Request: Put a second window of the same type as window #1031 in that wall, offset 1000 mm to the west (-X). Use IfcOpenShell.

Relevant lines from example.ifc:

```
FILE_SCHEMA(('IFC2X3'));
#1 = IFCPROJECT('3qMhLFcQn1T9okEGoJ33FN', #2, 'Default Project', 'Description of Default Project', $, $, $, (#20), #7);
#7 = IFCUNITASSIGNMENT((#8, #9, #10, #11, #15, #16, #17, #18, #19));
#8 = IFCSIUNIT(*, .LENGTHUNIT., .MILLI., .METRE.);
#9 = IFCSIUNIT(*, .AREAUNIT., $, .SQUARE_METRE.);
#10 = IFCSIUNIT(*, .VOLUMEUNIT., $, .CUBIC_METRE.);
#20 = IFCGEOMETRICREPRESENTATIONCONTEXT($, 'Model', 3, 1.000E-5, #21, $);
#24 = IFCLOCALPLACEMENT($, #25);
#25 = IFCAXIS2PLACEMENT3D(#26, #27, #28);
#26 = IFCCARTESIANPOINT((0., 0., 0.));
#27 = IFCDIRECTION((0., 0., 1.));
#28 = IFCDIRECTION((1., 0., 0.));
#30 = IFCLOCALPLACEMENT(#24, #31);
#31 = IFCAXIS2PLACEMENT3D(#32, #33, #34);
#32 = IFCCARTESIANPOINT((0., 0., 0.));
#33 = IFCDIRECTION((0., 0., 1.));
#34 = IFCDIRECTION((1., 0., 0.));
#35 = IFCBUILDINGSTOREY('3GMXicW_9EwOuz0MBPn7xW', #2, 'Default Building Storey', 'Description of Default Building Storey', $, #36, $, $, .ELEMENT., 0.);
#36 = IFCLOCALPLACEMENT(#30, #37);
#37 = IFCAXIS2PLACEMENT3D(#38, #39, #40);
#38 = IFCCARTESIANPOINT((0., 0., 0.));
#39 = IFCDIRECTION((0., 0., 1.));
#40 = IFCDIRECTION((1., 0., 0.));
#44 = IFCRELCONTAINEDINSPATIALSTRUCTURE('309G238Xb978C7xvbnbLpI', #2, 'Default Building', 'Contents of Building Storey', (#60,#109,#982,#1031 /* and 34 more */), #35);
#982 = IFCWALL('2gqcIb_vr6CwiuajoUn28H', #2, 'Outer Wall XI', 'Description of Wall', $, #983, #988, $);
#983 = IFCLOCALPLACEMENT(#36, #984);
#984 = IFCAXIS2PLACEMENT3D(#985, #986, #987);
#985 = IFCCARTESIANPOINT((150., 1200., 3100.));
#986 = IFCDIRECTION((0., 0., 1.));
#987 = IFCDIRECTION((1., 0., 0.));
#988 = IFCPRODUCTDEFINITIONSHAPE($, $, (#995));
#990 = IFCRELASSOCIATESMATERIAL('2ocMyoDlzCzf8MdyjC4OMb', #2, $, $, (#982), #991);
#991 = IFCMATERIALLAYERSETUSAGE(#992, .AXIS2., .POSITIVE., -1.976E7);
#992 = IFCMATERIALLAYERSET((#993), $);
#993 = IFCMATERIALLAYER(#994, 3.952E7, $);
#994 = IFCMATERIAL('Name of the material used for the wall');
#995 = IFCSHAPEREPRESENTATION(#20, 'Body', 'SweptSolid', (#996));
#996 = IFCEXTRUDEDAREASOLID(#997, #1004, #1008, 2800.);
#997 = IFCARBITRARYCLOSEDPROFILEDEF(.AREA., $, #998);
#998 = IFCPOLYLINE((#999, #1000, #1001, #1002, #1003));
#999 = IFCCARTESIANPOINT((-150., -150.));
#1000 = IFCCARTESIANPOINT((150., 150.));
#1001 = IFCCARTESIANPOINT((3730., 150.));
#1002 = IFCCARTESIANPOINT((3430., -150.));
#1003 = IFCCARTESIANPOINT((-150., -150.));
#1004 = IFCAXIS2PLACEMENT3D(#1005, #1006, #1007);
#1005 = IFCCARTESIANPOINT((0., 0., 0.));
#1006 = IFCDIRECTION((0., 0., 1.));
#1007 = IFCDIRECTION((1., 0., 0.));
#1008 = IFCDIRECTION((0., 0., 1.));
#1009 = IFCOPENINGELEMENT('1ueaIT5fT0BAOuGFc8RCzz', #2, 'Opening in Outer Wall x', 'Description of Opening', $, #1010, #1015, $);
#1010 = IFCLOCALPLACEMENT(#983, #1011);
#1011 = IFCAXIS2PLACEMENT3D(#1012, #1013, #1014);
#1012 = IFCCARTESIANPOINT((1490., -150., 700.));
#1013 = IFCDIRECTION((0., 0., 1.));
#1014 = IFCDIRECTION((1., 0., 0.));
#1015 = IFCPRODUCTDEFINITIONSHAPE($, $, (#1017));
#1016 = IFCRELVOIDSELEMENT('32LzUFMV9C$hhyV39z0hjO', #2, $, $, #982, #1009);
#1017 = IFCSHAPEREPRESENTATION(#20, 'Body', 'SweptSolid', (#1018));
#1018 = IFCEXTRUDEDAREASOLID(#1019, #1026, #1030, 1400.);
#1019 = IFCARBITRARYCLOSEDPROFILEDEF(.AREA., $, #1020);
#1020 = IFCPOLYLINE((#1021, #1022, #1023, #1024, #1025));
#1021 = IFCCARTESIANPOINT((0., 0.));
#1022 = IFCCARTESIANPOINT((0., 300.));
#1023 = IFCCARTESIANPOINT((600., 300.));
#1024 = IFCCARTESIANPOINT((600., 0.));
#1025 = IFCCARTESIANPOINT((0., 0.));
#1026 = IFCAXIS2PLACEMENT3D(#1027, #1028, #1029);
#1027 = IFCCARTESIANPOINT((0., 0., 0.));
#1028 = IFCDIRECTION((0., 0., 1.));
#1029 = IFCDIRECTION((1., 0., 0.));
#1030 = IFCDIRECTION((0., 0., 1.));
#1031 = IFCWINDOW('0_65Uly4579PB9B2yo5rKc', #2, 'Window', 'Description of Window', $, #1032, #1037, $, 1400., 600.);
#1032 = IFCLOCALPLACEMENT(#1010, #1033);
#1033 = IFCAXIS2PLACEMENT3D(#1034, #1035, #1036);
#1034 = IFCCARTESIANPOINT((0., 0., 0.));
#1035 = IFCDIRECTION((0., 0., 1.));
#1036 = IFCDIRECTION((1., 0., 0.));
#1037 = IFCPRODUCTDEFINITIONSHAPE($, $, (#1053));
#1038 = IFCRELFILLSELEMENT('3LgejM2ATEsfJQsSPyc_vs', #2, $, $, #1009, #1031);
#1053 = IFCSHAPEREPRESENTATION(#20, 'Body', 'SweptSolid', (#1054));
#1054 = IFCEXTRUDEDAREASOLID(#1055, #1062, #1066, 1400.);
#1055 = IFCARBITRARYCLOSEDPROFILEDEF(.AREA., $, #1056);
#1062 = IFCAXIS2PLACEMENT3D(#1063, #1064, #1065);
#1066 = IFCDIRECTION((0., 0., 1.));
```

```python
import ifcopenshell
import ifcopenshell.api.feature
import ifcopenshell.api.geometry
import ifcopenshell.api.root
import ifcopenshell.geom
import ifcopenshell.util.element
import ifcopenshell.util.placement
import ifcopenshell.util.shape
import ifcopenshell.util.unit

model = ifcopenshell.open("example.ifc")
unit_scale = ifcopenshell.util.unit.calculate_unit_scale(model)
settings = ifcopenshell.geom.settings()


def volume(element):
    """Net volume in cubic metres, openings subtracted."""
    shape = ifcopenshell.geom.create_shape(settings, element)
    return ifcopenshell.util.shape.get_volume(shape.geometry)


def reuse_history(source, copy):
    """copy_class also copies each property set's owner history, people and application; keep the originals."""
    for rel in copy.IsDefinedBy:
        if rel.is_a("IfcRelDefinesByProperties") and (history := rel.RelatingPropertyDefinition.OwnerHistory):
            rel.RelatingPropertyDefinition.OwnerHistory = source.OwnerHistory
            ifcopenshell.util.element.remove_deep2(model, history)


window = model.by_guid("0_65Uly4579PB9B2yo5rKc")
opening = window.FillsVoids[0].RelatingOpeningElement
wall = opening.VoidsElements[0].RelatingBuildingElement
before = volume(wall)
shift = ifcopenshell.util.placement.get_local_placement(wall.ObjectPlacement)[:3, 0] * -1 / unit_scale

# copy_class copies the void relationship, type, container and properties, but no geometry.
new_opening = ifcopenshell.api.root.copy_class(model, product=opening)
new_opening.Representation = ifcopenshell.util.element.copy_deep(
    model, opening.Representation, exclude=["IfcGeometricRepresentationContext", "IfcRepresentationMap"]
)
new_window = ifcopenshell.api.root.copy_class(model, product=window)
new_window.Representation = ifcopenshell.util.element.copy_deep(
    model, window.Representation, exclude=["IfcGeometricRepresentationContext", "IfcRepresentationMap"]
)
reuse_history(window, new_window)
fills = ifcopenshell.api.feature.add_filling(model, opening=new_opening, element=new_window)
fills.OwnerHistory = new_window.OwnerHistory  # required in IFC2X3

for old, new in ((opening, new_opening), (window, new_window)):
    matrix = ifcopenshell.util.placement.get_local_placement(old.ObjectPlacement)
    matrix[:3, 3] += shift
    ifcopenshell.api.geometry.edit_object_placement(model, product=new, matrix=matrix, is_si=False)

after = volume(wall)

print(f"wall volume {before:.3f} -> {after:.3f} m3")

model.write("example_edited.ifc")
```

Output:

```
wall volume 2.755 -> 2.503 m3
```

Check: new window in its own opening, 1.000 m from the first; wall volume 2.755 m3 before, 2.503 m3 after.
